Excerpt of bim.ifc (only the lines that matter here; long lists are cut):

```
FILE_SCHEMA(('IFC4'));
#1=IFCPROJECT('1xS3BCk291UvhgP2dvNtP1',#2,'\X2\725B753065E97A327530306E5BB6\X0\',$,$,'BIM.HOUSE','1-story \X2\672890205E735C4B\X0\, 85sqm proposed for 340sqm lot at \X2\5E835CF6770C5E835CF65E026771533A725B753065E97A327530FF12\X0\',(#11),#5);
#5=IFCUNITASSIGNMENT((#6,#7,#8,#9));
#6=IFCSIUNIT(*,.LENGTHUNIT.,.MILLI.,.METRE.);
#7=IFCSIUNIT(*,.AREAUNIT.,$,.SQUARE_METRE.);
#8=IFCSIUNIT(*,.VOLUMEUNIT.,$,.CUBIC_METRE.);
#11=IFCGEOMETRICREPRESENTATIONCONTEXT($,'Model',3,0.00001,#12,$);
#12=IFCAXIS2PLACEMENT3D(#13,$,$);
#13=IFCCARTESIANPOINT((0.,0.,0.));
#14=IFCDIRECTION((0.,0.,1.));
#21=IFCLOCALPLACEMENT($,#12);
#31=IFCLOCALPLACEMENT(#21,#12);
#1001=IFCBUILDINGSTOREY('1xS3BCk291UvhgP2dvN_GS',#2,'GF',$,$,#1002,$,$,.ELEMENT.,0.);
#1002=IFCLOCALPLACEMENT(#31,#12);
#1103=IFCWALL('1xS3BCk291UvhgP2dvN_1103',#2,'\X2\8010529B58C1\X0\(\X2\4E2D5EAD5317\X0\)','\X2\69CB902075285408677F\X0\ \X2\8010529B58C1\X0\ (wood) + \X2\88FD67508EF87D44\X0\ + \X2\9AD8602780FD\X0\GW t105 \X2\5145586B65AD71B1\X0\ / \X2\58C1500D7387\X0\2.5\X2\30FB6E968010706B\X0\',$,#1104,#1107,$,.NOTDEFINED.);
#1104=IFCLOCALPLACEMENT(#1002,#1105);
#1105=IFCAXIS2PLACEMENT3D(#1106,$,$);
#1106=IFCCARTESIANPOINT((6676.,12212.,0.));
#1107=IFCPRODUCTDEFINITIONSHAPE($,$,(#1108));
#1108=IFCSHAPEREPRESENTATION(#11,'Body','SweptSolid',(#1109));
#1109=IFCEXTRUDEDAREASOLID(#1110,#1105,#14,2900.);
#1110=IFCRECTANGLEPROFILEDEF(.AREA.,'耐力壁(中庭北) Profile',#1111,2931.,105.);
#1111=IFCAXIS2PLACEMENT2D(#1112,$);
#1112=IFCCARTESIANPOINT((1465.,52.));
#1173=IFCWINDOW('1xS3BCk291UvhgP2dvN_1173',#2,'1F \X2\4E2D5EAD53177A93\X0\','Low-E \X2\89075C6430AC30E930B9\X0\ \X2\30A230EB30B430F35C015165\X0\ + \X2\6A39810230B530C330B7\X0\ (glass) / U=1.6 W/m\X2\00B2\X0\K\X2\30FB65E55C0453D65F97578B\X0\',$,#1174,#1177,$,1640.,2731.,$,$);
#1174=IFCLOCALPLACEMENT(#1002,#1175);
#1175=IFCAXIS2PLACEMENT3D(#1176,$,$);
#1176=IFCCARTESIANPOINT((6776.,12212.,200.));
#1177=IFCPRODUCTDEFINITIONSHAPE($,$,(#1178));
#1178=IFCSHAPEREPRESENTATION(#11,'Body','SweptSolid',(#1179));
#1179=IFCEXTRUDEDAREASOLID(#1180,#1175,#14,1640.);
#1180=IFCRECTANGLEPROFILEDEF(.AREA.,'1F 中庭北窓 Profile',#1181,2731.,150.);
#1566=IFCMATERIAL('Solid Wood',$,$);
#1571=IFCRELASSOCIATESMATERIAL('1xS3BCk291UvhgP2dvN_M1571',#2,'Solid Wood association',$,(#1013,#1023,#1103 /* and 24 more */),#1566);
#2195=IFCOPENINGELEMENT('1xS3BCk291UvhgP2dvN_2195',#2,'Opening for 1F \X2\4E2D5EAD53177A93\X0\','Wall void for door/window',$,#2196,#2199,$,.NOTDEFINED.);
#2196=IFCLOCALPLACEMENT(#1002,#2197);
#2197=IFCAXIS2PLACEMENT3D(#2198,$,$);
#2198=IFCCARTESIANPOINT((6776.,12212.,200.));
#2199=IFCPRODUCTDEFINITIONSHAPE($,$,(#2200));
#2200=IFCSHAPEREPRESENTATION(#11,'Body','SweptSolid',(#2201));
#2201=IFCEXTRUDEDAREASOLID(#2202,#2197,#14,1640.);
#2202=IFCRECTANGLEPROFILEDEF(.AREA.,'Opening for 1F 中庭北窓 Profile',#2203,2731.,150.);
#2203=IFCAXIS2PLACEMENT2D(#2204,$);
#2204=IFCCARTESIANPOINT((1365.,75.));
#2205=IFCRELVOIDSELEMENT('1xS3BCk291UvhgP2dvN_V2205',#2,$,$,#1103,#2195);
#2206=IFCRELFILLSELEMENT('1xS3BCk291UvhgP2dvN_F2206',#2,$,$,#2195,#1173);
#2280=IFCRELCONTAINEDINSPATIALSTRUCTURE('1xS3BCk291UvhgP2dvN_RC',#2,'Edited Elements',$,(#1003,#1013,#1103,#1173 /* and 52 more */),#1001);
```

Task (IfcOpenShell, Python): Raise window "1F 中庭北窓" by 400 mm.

```python
import numpy as np
import ifcopenshell
import ifcopenshell.api.geometry
import ifcopenshell.util.placement
import ifcopenshell.util.unit

model = ifcopenshell.open("bim.ifc")
unit_scale = ifcopenshell.util.unit.calculate_unit_scale(model)

window = model.by_guid("1xS3BCk291UvhgP2dvN_1173")
opening = window.FillsVoids[0].RelatingOpeningElement
dz = 0.4 / unit_scale

shift = np.array([0.0, 0.0, dz])
# The window is not placed relative to its opening, so move both.
for product in (opening, window):
    matrix = ifcopenshell.util.placement.get_local_placement(product.ObjectPlacement)
    matrix[:3, 3] += shift
    ifcopenshell.api.geometry.edit_object_placement(model, product=product, matrix=matrix, is_si=False)

print(f"moved by {dz * unit_scale:+.3f} m")

model.write("bim_updated.ifc")
```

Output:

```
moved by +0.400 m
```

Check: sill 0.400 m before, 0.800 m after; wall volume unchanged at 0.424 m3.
